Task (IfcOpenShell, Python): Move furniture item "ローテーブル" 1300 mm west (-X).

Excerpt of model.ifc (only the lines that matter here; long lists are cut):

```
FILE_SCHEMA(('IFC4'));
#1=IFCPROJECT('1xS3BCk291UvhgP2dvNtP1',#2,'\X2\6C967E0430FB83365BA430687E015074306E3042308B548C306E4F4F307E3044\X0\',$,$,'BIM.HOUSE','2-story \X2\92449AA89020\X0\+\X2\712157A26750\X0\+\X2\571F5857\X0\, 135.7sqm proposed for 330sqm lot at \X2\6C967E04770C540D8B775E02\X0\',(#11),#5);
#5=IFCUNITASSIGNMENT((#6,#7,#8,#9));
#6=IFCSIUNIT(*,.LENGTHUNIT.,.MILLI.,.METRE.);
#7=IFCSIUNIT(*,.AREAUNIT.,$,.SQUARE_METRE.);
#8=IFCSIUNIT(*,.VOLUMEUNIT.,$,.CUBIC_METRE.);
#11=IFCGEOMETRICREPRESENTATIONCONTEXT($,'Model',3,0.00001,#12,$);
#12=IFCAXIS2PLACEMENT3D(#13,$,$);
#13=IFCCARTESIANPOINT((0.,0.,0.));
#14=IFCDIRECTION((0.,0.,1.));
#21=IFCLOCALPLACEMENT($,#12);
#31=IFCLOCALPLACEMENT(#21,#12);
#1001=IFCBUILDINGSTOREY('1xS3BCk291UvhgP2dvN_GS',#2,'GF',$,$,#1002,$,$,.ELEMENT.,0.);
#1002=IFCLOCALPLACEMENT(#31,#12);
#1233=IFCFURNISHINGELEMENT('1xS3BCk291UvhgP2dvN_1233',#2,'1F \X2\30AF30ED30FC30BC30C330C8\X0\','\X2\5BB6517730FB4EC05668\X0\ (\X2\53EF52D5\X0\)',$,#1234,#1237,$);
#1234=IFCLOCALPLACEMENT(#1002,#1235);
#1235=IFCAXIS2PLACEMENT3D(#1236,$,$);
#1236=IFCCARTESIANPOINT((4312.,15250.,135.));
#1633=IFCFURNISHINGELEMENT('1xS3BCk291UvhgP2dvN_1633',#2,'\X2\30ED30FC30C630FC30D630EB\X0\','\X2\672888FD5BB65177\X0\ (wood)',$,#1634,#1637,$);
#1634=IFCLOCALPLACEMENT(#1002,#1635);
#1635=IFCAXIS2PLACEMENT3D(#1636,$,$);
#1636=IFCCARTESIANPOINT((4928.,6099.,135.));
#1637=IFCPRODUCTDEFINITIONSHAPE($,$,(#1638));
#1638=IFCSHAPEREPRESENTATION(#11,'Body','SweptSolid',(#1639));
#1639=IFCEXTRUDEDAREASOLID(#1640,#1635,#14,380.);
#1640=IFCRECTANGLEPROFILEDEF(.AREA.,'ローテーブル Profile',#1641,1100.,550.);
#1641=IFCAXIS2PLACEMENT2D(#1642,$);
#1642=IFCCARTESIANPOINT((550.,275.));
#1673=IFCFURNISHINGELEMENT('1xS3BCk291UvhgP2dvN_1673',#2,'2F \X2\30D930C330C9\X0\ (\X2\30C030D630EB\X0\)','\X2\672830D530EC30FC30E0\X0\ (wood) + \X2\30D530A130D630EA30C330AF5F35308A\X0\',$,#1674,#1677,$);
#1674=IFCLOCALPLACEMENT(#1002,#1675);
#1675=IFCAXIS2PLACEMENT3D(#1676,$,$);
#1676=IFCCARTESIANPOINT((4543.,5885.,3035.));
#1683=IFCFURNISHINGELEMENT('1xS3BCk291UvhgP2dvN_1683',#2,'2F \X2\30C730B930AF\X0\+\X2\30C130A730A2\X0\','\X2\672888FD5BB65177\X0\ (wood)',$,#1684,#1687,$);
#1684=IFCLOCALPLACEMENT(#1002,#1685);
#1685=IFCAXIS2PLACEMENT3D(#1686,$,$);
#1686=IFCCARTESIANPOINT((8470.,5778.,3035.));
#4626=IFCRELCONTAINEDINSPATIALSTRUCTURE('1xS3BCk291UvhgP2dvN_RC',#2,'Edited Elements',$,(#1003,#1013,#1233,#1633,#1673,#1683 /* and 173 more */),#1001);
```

```python
import ifcopenshell
import ifcopenshell.api.geometry
import ifcopenshell.util.placement
import ifcopenshell.util.unit

model = ifcopenshell.open("model.ifc")
unit_scale = ifcopenshell.util.unit.calculate_unit_scale(model)

item = model.by_guid("1xS3BCk291UvhgP2dvN_1633")
matrix = ifcopenshell.util.placement.get_local_placement(item.ObjectPlacement)
matrix[0, 3] -= 1.3 / unit_scale
ifcopenshell.api.geometry.edit_object_placement(model, product=item, matrix=matrix, is_si=False)

print(ifcopenshell.util.placement.get_local_placement(item.ObjectPlacement).round(3) + 0.0)

model.write("model_updated.ifc")
```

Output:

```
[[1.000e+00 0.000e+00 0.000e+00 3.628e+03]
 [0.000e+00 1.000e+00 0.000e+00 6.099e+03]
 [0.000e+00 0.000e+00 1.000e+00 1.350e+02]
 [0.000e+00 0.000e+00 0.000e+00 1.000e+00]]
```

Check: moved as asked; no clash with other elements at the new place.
